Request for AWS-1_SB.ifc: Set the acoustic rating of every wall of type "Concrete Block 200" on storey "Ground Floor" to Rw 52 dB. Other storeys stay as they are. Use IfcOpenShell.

First a look at what the model holds.

```python
import ifcopenshell
import ifcopenshell.util.element

model = ifcopenshell.open("AWS-1_SB.ifc")
print(model.schema)
storey = next(s for s in model.by_type("IfcBuildingStorey") if s.Name == "Ground Floor")
walls = [e for e in ifcopenshell.util.element.get_decomposition(storey) if e.is_a("IfcWall")]
seen = {}
for e in walls:
    element_type = ifcopenshell.util.element.get_type(e)
    key = (element_type.Name if element_type != e and element_type else None, ifcopenshell.util.element.get_pset(e, "Pset_WallCommon", "AcousticRating"))
    seen[key] = seen.get(key, 0) + 1
for (name, value), count in sorted(seen.items(), key=str):
    print(count, "x", name, "|", value)
```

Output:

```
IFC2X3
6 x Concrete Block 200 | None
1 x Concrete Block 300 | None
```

```python
import ifcopenshell
import ifcopenshell.api.pset
import ifcopenshell.util.element

model = ifcopenshell.open("AWS-1_SB.ifc")

storey = next(s for s in model.by_type("IfcBuildingStorey") if s.Name == "Ground Floor")
walls = [e for e in ifcopenshell.util.element.get_decomposition(storey) if e.is_a("IfcWall")]

count = 0
for e in walls:
    element_type = ifcopenshell.util.element.get_type(e)
    if element_type in (None, e) or element_type.Name != "Concrete Block 200":
        continue
    # add_pset returns the element's existing set when there is one.
    pset = ifcopenshell.api.pset.add_pset(model, product=e, name="Pset_WallCommon")
    ifcopenshell.api.pset.edit_pset(model, pset=pset, properties={"AcousticRating": "Rw 52 dB"})
    count += 1

print(count, "walls updated")

model.write("AWS-1_SB_updated.ifc")
```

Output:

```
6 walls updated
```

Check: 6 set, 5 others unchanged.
